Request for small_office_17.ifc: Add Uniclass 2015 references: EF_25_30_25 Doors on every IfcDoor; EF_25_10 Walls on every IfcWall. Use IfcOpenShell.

First a look at what the model holds.

```python
import ifcopenshell

model = ifcopenshell.open("small_office_17.ifc")
print(model.schema)
print("classifications:", [c.Name for c in model.by_type("IfcClassification")])
for ifc_class in ("IfcDoor", "IfcRoof", "IfcStair", "IfcWall", "IfcWindow"):
    print(ifc_class, len(model.by_type(ifc_class)))
```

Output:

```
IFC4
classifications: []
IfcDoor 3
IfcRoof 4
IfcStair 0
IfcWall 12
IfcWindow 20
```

```python
import ifcopenshell
import ifcopenshell.api.classification

model = ifcopenshell.open("small_office_17.ifc")

system = ifcopenshell.api.classification.add_classification(model, classification="Uniclass 2015")

codes = {
    "IfcDoor": ("EF_25_30_25", "Doors"),
    "IfcWall": ("EF_25_10", "Walls"),
}
for ifc_class, (code, name) in codes.items():
    products = model.by_type(ifc_class)
    ifcopenshell.api.classification.add_reference(
        model, products=products, classification=system, identification=code, name=name
    )
    print(code, len(products))

model.write("small_office_17_rev.ifc")
```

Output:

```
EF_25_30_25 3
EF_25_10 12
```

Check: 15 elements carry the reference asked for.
